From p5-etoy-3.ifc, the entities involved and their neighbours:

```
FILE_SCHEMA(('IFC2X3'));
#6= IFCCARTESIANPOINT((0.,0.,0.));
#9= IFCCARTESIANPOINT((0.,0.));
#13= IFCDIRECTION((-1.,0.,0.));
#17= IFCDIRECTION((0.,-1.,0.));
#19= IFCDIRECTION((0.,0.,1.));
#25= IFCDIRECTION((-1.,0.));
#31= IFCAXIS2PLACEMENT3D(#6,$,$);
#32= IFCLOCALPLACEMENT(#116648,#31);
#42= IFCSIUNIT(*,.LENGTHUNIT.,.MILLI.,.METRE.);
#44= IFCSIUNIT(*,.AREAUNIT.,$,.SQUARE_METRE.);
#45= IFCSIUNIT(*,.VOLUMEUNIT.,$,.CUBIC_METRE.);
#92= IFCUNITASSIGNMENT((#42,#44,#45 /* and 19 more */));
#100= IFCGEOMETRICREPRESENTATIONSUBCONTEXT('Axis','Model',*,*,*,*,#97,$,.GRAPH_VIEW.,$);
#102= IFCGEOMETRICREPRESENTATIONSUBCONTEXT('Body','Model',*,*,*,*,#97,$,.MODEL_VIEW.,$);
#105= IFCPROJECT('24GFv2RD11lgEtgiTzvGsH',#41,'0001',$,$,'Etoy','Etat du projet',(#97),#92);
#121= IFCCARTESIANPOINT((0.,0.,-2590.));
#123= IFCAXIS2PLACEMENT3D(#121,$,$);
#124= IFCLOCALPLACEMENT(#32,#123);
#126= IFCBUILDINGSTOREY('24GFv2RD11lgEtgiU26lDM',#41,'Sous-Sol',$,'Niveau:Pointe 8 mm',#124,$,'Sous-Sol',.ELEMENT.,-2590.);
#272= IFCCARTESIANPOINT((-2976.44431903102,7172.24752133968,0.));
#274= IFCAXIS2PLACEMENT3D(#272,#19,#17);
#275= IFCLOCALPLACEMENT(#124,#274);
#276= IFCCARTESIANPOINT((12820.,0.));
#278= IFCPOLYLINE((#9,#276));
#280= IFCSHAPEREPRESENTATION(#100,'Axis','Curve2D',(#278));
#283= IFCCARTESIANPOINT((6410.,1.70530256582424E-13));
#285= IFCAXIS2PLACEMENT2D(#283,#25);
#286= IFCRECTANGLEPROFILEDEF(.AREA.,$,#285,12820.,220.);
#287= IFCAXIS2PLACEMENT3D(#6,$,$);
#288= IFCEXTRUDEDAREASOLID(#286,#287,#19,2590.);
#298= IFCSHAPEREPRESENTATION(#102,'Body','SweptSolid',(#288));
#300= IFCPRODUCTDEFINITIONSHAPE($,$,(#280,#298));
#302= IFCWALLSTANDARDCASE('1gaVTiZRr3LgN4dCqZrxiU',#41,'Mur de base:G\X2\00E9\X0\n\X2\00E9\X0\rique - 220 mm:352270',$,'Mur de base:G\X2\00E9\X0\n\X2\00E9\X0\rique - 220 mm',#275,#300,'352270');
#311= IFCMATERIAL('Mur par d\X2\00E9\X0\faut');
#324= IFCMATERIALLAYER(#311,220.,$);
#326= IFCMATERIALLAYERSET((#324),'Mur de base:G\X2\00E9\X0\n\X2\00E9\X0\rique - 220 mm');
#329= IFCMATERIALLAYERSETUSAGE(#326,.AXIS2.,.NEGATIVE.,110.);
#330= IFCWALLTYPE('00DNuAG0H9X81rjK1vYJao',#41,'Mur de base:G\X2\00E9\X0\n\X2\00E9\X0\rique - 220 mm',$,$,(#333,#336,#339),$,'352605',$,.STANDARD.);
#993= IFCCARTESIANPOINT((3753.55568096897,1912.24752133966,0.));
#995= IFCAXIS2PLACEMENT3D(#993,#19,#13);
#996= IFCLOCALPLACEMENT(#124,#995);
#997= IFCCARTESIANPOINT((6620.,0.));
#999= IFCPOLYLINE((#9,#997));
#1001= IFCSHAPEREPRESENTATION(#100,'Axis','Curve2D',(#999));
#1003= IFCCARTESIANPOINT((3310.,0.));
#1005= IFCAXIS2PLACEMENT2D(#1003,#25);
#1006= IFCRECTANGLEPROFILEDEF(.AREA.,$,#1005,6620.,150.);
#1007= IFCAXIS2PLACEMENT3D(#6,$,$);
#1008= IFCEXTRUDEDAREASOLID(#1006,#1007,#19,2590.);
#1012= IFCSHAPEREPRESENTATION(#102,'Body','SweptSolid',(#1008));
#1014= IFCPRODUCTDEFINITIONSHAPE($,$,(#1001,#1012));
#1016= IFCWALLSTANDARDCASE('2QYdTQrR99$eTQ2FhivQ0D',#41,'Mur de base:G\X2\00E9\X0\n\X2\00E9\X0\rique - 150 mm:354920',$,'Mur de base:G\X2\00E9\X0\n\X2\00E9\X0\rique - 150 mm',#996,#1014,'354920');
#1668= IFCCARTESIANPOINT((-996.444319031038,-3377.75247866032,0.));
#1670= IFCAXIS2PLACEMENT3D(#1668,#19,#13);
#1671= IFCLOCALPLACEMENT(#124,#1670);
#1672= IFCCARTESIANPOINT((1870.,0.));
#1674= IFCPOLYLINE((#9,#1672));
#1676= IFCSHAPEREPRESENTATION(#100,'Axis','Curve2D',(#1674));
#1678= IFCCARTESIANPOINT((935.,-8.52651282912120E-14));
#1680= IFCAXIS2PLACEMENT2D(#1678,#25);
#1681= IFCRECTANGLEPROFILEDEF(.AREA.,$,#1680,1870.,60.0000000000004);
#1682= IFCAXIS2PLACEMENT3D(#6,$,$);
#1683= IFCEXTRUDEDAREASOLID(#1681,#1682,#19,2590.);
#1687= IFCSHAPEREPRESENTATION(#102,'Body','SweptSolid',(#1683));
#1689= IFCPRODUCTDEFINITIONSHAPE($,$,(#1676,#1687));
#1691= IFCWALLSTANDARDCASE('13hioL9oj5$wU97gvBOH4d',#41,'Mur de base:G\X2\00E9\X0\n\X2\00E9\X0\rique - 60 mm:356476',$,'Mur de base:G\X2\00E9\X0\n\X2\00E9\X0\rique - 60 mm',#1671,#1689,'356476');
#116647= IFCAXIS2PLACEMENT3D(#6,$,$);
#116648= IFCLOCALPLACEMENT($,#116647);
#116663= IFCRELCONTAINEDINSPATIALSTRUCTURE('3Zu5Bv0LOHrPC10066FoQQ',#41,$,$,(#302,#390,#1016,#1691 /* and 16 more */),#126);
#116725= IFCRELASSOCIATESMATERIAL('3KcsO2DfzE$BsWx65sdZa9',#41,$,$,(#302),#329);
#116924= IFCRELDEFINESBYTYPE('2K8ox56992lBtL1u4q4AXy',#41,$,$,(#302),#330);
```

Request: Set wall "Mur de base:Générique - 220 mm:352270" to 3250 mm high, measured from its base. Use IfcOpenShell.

```python
import ifcopenshell
import ifcopenshell.geom
import ifcopenshell.util.representation
import ifcopenshell.util.shape
import ifcopenshell.util.unit

model = ifcopenshell.open("p5-etoy-3.ifc")
unit_scale = ifcopenshell.util.unit.calculate_unit_scale(model)
settings = ifcopenshell.geom.settings()


def volume(element):
    """Net volume in cubic metres, openings subtracted."""
    shape = ifcopenshell.geom.create_shape(settings, element)
    return ifcopenshell.util.shape.get_volume(shape.geometry)


wall = model.by_guid("1gaVTiZRr3LgN4dCqZrxiU")
before = volume(wall)

body = ifcopenshell.util.representation.get_representation(wall, "Model", "Body")
solid = body.Items[0]
old_height = solid.Depth
solid.Depth = 3.25 / unit_scale
after = volume(wall)

print(f"height {old_height:g} -> {solid.Depth:g}, volume {before:.3f} -> {after:.3f} m3")

model.write("p5-etoy-3_rev.ifc")
```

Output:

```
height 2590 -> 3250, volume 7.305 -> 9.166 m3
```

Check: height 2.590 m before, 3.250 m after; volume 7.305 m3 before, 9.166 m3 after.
